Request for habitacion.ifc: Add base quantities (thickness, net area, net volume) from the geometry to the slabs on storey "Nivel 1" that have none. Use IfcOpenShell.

First a look at what the model holds.

```python
import ifcopenshell
import ifcopenshell.util.element
import ifcopenshell.util.unit

model = ifcopenshell.open("habitacion.ifc")
print(model.schema)
for unit_type in ("LENGTHUNIT", "AREAUNIT", "VOLUMEUNIT"):
    print(unit_type, ifcopenshell.util.unit.calculate_unit_scale(model, unit_type))
storey = next(s for s in model.by_type("IfcBuildingStorey") if s.Name == "Nivel 1")
slabs = [e for e in ifcopenshell.util.element.get_decomposition(storey) if e.is_a("IfcSlab")]
for e in sorted(slabs, key=lambda e: e.id()):
    print(e.id(), e.is_a(), e.Name, list(ifcopenshell.util.element.get_psets(e, qtos_only=True)), sep=" | ")
```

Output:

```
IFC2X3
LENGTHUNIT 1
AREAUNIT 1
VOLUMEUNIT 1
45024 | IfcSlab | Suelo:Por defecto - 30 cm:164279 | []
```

```python
import ifcopenshell
import ifcopenshell.api.pset
import ifcopenshell.geom
import ifcopenshell.util.element
import ifcopenshell.util.shape
import ifcopenshell.util.unit

model = ifcopenshell.open("habitacion.ifc")
unit_scale = ifcopenshell.util.unit.calculate_unit_scale(model)
area_scale = ifcopenshell.util.unit.calculate_unit_scale(model, "AREAUNIT")
volume_scale = ifcopenshell.util.unit.calculate_unit_scale(model, "VOLUMEUNIT")
settings = ifcopenshell.geom.settings()

storey = next(s for s in model.by_type("IfcBuildingStorey") if s.Name == "Nivel 1")
slabs = [e for e in ifcopenshell.util.element.get_decomposition(storey) if e.is_a("IfcSlab")]

for e in sorted(slabs, key=lambda e: e.id()):
    if ifcopenshell.util.element.get_psets(e, qtos_only=True, should_inherit=False):
        continue
    # Geometry comes back in metres, in the element's own axes.
    shape = ifcopenshell.geom.create_shape(settings, e)
    values = {
        "Width": ifcopenshell.util.shape.get_z(shape.geometry) / unit_scale,
        "NetArea": ifcopenshell.util.shape.get_footprint_area(shape.geometry) / area_scale,
        "NetVolume": ifcopenshell.util.shape.get_volume(shape.geometry) / volume_scale,
    }
    qto = ifcopenshell.api.pset.add_qto(model, product=e, name="BaseQuantities")
    ifcopenshell.api.pset.edit_qto(model, qto=qto, properties=values)
    print(e.id(), {k: round(v, 3) for k, v in values.items()})

model.write("habitacion_rev.ifc")
```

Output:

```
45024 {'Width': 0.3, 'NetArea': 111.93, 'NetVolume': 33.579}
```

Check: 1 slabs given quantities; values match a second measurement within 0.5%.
